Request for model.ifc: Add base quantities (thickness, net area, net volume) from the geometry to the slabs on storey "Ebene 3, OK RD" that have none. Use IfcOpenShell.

First a look at what the model holds.

```python
import ifcopenshell
import ifcopenshell.util.element
import ifcopenshell.util.unit

model = ifcopenshell.open("model.ifc")
print(model.schema)
for unit_type in ("LENGTHUNIT", "AREAUNIT", "VOLUMEUNIT"):
    print(unit_type, ifcopenshell.util.unit.calculate_unit_scale(model, unit_type))
storey = next(s for s in model.by_type("IfcBuildingStorey") if s.Name == "Ebene 3, OK RD")
slabs = [e for e in ifcopenshell.util.element.get_decomposition(storey) if e.is_a("IfcSlab")]
for e in sorted(slabs, key=lambda e: e.id()):
    print(e.id(), e.is_a(), e.Name, list(ifcopenshell.util.element.get_psets(e, qtos_only=True)), sep=" | ")
```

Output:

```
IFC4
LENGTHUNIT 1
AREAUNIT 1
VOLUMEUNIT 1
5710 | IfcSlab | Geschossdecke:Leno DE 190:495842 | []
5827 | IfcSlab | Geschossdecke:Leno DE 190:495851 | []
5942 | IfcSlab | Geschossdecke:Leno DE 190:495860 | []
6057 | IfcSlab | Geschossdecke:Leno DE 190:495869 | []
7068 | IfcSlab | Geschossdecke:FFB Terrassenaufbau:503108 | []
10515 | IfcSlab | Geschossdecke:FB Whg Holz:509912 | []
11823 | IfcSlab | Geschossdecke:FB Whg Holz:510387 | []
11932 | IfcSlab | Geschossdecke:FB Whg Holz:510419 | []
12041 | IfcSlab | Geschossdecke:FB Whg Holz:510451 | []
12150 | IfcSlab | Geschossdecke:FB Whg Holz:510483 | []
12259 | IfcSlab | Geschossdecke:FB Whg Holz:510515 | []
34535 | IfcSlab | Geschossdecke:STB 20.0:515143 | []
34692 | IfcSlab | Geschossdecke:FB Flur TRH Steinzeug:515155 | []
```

```python
import ifcopenshell
import ifcopenshell.api.pset
import ifcopenshell.geom
import ifcopenshell.util.element
import ifcopenshell.util.shape
import ifcopenshell.util.unit

model = ifcopenshell.open("model.ifc")
unit_scale = ifcopenshell.util.unit.calculate_unit_scale(model)
area_scale = ifcopenshell.util.unit.calculate_unit_scale(model, "AREAUNIT")
volume_scale = ifcopenshell.util.unit.calculate_unit_scale(model, "VOLUMEUNIT")
settings = ifcopenshell.geom.settings()

storey = next(s for s in model.by_type("IfcBuildingStorey") if s.Name == "Ebene 3, OK RD")
slabs = [e for e in ifcopenshell.util.element.get_decomposition(storey) if e.is_a("IfcSlab")]

for e in sorted(slabs, key=lambda e: e.id()):
    if ifcopenshell.util.element.get_psets(e, qtos_only=True, should_inherit=False):
        continue
    # Geometry comes back in metres, in the element's own axes.
    shape = ifcopenshell.geom.create_shape(settings, e)
    values = {
        "Width": ifcopenshell.util.shape.get_z(shape.geometry) / unit_scale,
        "NetArea": ifcopenshell.util.shape.get_footprint_area(shape.geometry) / area_scale,
        "NetVolume": ifcopenshell.util.shape.get_volume(shape.geometry) / volume_scale,
    }
    qto = ifcopenshell.api.pset.add_qto(model, product=e, name="Qto_SlabBaseQuantities")
    ifcopenshell.api.pset.edit_qto(model, qto=qto, properties=values)
    print(e.id(), {k: round(v, 3) for k, v in values.items()})

model.write("model_rev.ifc")
```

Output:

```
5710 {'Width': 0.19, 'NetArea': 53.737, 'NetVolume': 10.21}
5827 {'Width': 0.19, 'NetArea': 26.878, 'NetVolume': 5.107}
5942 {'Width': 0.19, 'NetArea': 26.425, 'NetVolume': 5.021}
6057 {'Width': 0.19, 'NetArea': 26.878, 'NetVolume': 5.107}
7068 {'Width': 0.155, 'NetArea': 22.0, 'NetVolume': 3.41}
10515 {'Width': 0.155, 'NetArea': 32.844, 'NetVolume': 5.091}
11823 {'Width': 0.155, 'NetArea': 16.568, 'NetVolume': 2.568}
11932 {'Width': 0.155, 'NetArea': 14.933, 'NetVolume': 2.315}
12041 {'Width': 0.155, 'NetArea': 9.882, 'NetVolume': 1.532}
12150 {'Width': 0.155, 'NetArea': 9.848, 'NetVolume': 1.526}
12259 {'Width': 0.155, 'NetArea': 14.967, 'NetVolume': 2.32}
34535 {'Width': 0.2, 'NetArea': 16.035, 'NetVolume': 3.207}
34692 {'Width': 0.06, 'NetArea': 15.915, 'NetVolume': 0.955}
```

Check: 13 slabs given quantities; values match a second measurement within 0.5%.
